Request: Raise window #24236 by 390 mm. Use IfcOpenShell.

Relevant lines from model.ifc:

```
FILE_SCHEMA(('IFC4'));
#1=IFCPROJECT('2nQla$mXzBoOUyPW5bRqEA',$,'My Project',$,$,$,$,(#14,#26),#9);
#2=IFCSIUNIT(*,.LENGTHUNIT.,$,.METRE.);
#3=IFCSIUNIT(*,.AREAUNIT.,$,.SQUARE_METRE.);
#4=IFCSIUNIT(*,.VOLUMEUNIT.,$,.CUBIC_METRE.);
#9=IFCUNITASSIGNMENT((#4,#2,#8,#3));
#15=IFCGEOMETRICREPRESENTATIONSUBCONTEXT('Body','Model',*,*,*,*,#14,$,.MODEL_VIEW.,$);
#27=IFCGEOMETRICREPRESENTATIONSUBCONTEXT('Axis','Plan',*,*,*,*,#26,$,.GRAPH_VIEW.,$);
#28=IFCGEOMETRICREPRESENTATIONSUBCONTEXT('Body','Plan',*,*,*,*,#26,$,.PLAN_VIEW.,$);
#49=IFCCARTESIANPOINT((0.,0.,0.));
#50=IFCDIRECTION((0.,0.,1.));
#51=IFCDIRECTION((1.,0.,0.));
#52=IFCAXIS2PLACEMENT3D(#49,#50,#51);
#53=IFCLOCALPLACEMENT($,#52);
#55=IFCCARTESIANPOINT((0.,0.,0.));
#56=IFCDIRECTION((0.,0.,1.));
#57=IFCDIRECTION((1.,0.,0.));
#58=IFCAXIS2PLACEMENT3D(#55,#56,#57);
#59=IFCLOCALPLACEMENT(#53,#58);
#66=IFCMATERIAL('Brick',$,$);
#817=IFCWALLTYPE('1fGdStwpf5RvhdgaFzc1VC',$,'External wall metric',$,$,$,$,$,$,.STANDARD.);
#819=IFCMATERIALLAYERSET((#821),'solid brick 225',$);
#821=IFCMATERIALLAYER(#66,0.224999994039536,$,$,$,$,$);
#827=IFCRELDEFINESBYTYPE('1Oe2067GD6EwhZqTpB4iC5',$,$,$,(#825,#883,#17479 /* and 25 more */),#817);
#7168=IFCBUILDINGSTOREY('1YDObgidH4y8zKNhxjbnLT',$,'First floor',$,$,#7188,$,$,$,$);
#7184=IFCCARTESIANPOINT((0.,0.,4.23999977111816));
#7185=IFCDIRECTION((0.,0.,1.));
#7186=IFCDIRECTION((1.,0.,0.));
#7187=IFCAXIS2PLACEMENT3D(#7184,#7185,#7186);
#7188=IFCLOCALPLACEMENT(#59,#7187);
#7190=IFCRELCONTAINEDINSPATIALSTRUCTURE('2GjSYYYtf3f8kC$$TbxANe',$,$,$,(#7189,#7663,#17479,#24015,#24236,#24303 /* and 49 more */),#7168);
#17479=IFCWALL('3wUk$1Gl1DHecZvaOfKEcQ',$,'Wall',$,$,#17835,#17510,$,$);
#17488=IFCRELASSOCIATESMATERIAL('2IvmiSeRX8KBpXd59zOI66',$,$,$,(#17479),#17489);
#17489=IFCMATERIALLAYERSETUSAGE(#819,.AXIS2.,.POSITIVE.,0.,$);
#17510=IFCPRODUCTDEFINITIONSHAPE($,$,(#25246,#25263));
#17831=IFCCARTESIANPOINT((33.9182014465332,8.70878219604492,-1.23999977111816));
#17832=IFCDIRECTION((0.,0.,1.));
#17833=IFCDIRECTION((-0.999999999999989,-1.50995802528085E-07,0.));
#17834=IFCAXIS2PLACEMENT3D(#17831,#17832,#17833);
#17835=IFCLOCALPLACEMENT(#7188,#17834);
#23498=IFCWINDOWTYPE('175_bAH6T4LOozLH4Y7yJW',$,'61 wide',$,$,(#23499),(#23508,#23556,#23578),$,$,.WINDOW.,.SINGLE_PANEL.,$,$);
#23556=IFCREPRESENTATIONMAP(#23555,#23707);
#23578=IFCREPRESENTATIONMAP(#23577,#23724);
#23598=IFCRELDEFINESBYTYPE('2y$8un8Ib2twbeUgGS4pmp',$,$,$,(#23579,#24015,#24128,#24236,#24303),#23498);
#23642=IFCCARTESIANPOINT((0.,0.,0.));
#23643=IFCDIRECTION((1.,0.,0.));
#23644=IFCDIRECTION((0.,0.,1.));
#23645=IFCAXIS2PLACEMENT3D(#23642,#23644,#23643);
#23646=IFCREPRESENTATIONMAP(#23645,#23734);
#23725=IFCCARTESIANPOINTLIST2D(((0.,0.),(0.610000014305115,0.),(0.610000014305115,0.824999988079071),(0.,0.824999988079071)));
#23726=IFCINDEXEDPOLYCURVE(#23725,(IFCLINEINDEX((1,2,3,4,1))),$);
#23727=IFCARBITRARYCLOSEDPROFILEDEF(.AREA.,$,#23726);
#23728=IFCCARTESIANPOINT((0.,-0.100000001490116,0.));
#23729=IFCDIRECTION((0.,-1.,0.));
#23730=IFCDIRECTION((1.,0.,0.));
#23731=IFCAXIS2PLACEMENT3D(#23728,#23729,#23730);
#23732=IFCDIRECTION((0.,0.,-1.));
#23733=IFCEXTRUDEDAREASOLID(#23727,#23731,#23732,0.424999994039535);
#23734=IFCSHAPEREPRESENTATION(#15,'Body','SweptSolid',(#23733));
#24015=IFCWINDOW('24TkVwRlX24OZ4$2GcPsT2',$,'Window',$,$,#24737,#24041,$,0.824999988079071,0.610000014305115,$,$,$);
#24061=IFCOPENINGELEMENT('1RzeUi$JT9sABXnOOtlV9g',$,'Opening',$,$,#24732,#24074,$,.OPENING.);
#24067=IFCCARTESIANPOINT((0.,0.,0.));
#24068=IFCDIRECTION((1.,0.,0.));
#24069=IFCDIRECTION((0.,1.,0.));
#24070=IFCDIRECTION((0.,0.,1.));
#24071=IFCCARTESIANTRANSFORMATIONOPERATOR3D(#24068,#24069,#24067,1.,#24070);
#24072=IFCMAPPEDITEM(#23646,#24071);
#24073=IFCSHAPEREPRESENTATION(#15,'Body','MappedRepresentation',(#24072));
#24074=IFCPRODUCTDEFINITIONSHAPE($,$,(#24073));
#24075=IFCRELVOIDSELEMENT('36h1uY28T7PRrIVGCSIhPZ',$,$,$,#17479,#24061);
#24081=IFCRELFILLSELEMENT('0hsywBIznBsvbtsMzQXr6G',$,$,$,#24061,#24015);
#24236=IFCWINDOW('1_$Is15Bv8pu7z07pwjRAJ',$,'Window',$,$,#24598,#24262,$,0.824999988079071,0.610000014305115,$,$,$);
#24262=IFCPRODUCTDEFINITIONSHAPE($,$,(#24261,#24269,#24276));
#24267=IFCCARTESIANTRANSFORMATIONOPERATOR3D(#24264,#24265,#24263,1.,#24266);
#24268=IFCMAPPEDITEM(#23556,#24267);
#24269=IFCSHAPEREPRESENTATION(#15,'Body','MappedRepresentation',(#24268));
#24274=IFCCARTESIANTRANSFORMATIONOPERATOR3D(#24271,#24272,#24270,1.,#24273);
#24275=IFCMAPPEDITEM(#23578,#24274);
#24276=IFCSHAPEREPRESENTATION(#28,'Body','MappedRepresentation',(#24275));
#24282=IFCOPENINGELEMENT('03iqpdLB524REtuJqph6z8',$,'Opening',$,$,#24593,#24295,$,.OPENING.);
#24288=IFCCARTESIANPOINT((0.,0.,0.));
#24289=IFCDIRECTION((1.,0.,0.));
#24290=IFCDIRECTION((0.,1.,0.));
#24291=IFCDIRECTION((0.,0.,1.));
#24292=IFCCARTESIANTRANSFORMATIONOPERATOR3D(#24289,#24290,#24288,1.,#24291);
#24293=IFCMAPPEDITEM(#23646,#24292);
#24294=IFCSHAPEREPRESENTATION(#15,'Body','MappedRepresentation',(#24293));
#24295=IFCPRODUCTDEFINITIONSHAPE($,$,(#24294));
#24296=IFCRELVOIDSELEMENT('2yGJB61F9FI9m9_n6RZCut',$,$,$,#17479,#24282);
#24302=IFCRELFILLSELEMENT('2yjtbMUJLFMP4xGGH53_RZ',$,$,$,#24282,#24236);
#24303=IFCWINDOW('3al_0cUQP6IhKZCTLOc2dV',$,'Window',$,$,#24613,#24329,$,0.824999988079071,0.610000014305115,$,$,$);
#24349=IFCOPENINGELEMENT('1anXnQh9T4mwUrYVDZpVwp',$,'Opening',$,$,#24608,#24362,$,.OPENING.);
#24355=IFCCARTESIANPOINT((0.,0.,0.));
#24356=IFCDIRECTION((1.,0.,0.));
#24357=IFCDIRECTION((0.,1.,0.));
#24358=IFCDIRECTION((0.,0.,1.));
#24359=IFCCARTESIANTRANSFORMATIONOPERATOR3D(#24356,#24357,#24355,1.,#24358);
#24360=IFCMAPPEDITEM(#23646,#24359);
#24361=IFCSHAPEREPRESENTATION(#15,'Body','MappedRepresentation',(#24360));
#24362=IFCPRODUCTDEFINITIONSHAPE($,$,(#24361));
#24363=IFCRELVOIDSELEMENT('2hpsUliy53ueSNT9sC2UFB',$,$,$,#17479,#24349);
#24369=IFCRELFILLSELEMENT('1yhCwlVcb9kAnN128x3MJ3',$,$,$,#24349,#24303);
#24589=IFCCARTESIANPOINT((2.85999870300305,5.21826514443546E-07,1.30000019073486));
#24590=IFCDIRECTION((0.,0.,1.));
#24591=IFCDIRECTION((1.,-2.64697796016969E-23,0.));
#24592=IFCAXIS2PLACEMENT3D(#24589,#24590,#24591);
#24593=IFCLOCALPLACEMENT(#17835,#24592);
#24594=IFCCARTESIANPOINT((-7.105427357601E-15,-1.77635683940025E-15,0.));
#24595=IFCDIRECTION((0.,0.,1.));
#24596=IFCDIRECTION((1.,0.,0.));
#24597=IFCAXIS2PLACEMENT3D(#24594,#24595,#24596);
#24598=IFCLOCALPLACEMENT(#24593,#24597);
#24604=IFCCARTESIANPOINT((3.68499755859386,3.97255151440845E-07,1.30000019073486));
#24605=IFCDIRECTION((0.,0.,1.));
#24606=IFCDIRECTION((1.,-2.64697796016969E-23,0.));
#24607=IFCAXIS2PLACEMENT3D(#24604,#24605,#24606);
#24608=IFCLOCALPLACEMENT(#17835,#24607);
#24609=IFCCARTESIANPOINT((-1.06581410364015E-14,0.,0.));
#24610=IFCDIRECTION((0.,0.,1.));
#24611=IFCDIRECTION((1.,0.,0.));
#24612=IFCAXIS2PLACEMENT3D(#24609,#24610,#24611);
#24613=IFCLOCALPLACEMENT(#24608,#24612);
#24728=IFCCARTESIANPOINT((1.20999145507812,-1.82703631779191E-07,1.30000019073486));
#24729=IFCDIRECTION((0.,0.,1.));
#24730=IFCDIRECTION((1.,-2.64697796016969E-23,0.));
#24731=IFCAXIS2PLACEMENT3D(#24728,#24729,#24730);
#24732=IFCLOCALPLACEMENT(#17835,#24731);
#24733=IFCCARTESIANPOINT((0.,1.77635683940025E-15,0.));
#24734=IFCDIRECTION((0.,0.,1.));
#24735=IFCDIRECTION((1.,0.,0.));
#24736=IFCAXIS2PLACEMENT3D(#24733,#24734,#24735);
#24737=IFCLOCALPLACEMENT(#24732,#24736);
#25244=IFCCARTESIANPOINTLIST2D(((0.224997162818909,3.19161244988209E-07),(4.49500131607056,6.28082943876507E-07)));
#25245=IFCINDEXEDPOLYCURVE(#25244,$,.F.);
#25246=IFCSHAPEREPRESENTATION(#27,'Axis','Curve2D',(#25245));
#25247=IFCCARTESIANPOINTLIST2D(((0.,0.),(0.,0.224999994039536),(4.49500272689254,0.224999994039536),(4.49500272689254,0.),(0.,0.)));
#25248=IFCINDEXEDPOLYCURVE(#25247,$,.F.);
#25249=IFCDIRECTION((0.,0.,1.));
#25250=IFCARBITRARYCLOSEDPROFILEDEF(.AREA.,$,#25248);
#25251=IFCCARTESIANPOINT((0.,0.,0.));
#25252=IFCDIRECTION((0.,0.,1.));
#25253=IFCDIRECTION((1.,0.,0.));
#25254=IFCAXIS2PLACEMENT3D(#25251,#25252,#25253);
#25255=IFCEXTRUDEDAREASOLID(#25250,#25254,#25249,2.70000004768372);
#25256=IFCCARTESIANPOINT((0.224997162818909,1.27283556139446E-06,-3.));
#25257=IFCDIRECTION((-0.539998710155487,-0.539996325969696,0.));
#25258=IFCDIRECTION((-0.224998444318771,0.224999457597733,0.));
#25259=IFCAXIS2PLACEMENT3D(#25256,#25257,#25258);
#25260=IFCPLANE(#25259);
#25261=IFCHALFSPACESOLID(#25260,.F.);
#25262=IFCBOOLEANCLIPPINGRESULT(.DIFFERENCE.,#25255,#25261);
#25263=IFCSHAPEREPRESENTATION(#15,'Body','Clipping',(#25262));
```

```python
import numpy as np
import ifcopenshell
import ifcopenshell.api.geometry
import ifcopenshell.util.placement
import ifcopenshell.util.unit

model = ifcopenshell.open("model.ifc")
unit_scale = ifcopenshell.util.unit.calculate_unit_scale(model)

window = model.by_guid("1_$Is15Bv8pu7z07pwjRAJ")
opening = window.FillsVoids[0].RelatingOpeningElement
dz = 0.39 / unit_scale

shift = np.array([0.0, 0.0, dz])
# The window is placed relative to its opening, so it follows when the opening moves.
matrix = ifcopenshell.util.placement.get_local_placement(opening.ObjectPlacement)
matrix[:3, 3] += shift
ifcopenshell.api.geometry.edit_object_placement(
    model, product=opening, matrix=matrix, is_si=False, should_transform_children=True
)

print(f"moved by {dz * unit_scale:+.3f} m")

model.write("model-out.ifc")
```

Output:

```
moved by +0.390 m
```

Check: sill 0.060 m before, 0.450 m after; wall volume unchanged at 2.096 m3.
